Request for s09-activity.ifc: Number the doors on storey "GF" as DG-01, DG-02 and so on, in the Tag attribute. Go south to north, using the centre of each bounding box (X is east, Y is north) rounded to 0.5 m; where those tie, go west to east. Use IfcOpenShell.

First a look at what the model holds.

```python
import ifcopenshell
import ifcopenshell.util.element
import ifcopenshell.util.placement

model = ifcopenshell.open("s09-activity.ifc")
print(model.schema)
storey = next(s for s in model.by_type("IfcBuildingStorey") if s.Name == "GF")
doors = [e for e in ifcopenshell.util.element.get_decomposition(storey) if e.is_a("IfcDoor")]
for e in sorted(doors, key=lambda e: e.id()):
    origin = ifcopenshell.util.placement.get_local_placement(e.ObjectPlacement)[:3, 3]
    print(e.id(), e.Tag, e.Name, origin.round(2) + 0.0, sep=" | ")
```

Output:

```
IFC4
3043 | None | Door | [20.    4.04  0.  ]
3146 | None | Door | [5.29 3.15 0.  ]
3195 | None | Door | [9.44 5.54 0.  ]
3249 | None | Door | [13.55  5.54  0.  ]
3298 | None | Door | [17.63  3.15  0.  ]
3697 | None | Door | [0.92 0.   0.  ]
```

```python
import ifcopenshell
import ifcopenshell.geom
import ifcopenshell.util.element
import ifcopenshell.util.shape

model = ifcopenshell.open("s09-activity.ifc")
settings = ifcopenshell.geom.settings()
settings.set("use-world-coords", True)


def centre(element):
    shape = ifcopenshell.geom.create_shape(settings, element)
    return ifcopenshell.util.shape.get_bbox_centroid(shape.geometry)


storey = next(s for s in model.by_type("IfcBuildingStorey") if s.Name == "GF")
doors = [e for e in ifcopenshell.util.element.get_decomposition(storey) if e.is_a("IfcDoor")]

# Insertion points can sit at a corner or the storey origin, so sort by the geometry (in metres).
centres = {e: centre(e) for e in doors}
doors.sort(key=lambda e: (round(centres[e][1] / 0.5), centres[e][0]))

for i, e in enumerate(doors, start=1):
    number = f"DG-{i:02d}"
    e.Tag = number
    print(e.id(), number)

model.write("s09-activity_rev.ifc")
```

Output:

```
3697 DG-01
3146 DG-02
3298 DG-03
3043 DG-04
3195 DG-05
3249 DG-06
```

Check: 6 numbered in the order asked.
